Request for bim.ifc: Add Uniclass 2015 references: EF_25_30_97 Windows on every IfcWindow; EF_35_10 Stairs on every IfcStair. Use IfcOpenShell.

First a look at what the model holds.

```python
import ifcopenshell

model = ifcopenshell.open("bim.ifc")
print(model.schema)
print("classifications:", [c.Name for c in model.by_type("IfcClassification")])
for ifc_class in ("IfcDoor", "IfcRoof", "IfcStair", "IfcWall", "IfcWindow"):
    print(ifc_class, len(model.by_type(ifc_class)))
```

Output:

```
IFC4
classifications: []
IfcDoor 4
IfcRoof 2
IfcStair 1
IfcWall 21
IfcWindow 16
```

```python
import ifcopenshell
import ifcopenshell.api.classification

model = ifcopenshell.open("bim.ifc")

system = ifcopenshell.api.classification.add_classification(model, classification="Uniclass 2015")

codes = {
    "IfcWindow": ("EF_25_30_97", "Windows"),
    "IfcStair": ("EF_35_10", "Stairs"),
}
for ifc_class, (code, name) in codes.items():
    products = model.by_type(ifc_class)
    ifcopenshell.api.classification.add_reference(
        model, products=products, classification=system, identification=code, name=name
    )
    print(code, len(products))

model.write("bim_v2.ifc")
```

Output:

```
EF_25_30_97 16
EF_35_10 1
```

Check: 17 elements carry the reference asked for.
